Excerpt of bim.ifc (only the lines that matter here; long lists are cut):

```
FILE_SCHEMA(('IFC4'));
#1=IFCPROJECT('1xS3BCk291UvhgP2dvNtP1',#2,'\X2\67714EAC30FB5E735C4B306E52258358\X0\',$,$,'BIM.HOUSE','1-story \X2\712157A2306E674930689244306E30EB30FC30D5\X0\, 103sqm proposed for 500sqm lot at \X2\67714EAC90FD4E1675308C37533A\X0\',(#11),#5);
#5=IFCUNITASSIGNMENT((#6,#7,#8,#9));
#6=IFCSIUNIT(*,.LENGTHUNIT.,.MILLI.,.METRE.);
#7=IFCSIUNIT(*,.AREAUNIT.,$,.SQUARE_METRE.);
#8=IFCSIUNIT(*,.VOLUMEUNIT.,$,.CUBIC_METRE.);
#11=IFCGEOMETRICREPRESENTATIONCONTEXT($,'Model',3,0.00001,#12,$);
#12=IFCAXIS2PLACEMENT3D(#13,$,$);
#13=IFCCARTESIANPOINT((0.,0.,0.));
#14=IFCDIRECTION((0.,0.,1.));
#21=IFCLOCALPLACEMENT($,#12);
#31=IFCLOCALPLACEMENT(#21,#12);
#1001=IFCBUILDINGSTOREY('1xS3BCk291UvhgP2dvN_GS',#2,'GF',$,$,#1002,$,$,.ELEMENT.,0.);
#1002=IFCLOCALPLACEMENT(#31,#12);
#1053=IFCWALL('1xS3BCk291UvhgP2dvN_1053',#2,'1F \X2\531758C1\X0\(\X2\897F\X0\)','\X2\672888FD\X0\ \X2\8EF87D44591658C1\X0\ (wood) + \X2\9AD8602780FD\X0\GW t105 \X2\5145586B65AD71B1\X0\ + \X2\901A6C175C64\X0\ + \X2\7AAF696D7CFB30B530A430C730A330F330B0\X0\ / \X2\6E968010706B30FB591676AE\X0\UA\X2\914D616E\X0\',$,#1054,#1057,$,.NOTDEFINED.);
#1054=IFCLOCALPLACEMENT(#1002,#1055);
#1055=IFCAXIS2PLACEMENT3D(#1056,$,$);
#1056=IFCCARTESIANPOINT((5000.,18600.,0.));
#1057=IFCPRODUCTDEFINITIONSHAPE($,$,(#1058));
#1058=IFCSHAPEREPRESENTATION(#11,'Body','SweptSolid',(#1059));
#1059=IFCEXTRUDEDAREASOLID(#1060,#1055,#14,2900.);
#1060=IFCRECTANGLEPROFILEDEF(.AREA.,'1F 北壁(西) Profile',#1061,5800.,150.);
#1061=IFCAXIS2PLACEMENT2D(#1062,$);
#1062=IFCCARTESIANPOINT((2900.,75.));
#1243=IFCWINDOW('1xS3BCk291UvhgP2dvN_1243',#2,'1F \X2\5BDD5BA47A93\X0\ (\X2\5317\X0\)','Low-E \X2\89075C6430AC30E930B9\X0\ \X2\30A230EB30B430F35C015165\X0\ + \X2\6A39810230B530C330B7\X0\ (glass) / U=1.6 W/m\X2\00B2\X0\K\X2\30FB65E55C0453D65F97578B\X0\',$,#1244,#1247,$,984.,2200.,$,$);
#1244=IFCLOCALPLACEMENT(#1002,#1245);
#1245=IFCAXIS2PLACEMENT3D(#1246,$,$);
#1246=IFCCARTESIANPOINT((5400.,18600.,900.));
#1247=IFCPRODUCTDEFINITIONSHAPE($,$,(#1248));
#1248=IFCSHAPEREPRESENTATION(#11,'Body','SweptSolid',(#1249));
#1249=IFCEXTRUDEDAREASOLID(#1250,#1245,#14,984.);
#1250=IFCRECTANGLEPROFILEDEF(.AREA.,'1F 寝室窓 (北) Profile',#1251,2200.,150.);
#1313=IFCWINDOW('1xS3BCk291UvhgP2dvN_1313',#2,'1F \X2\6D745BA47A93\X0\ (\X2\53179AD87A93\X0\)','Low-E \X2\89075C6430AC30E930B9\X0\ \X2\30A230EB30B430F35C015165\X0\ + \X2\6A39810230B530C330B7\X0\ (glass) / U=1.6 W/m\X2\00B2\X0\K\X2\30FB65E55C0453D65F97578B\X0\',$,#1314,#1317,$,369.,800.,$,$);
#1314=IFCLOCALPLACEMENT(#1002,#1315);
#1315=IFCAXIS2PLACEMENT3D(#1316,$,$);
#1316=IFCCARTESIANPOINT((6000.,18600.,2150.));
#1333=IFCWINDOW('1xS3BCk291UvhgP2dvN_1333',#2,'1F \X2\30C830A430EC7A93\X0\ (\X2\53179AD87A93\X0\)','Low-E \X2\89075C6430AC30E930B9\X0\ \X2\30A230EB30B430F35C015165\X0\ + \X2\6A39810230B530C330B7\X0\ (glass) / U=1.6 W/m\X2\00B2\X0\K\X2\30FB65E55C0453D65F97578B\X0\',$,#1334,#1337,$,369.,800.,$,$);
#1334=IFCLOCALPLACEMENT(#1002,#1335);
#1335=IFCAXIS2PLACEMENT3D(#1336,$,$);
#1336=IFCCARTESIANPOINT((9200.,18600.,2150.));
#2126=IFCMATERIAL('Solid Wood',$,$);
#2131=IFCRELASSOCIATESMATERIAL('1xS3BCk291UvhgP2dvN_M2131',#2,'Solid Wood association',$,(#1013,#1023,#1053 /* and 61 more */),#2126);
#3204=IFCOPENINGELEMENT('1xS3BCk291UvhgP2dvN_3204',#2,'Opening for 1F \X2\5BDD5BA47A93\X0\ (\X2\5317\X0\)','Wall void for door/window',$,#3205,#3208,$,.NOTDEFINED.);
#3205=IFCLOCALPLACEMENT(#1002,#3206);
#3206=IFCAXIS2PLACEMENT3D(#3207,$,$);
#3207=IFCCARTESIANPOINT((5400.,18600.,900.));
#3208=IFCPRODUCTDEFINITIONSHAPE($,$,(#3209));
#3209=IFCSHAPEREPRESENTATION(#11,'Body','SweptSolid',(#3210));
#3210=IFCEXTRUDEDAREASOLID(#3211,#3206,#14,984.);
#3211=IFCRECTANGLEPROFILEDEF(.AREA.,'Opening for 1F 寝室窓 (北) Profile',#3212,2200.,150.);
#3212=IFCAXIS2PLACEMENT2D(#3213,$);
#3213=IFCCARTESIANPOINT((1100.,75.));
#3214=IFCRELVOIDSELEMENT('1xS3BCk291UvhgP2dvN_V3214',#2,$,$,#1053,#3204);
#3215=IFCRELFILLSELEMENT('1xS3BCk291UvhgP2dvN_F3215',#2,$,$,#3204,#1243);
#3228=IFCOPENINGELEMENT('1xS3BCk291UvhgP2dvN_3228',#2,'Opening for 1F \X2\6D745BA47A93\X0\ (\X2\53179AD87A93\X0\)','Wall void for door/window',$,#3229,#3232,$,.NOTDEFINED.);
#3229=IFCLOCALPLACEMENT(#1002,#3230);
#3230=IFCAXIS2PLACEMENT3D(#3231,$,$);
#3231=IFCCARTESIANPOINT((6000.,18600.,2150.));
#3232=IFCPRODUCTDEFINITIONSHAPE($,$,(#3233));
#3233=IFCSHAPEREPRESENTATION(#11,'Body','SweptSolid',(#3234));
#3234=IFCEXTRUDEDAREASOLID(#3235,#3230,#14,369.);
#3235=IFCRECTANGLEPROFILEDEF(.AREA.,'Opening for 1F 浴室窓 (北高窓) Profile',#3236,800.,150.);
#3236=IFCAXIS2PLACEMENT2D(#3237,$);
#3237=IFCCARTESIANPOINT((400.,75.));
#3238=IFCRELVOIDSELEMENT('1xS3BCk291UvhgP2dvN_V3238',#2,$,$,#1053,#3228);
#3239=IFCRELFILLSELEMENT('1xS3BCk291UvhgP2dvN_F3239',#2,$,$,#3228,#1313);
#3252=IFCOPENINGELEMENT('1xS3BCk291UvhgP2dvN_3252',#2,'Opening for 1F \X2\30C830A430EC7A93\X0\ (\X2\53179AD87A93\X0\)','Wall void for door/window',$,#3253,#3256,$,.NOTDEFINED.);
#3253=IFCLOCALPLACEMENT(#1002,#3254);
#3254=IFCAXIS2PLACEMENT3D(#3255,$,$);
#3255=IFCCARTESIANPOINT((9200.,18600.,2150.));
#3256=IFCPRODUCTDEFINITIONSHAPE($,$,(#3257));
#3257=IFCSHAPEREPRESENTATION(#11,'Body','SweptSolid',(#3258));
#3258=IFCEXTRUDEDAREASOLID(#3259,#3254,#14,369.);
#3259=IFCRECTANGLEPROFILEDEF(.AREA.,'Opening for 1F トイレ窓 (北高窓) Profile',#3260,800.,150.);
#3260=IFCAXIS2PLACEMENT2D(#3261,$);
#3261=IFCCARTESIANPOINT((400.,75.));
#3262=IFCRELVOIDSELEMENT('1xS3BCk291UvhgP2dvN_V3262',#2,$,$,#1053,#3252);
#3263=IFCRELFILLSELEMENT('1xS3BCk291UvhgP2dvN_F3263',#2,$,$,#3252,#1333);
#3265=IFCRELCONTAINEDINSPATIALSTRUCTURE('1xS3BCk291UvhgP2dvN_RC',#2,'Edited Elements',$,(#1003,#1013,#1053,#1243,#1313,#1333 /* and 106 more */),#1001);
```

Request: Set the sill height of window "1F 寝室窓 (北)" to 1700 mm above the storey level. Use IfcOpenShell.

```python
import numpy as np
import ifcopenshell
import ifcopenshell.api.geometry
import ifcopenshell.geom
import ifcopenshell.util.element
import ifcopenshell.util.placement
import ifcopenshell.util.shape
import ifcopenshell.util.unit

model = ifcopenshell.open("bim.ifc")
unit_scale = ifcopenshell.util.unit.calculate_unit_scale(model)

window = model.by_id(1243)
opening = window.FillsVoids[0].RelatingOpeningElement
storey = ifcopenshell.util.element.get_container(window, ifc_class="IfcBuildingStorey")
level = ifcopenshell.util.placement.get_local_placement(storey.ObjectPlacement)[2, 3]

# The opening's origin need not be at the sill, so measure its lowest point.
shape = ifcopenshell.geom.create_shape(ifcopenshell.geom.settings(), opening)
bottom = ifcopenshell.util.shape.get_shape_bottom_elevation(shape, shape.geometry) / unit_scale
dz = level + 1.7 / unit_scale - bottom

shift = np.array([0.0, 0.0, dz])
# The window is not placed relative to its opening, so move both.
for product in (opening, window):
    matrix = ifcopenshell.util.placement.get_local_placement(product.ObjectPlacement)
    matrix[:3, 3] += shift
    ifcopenshell.api.geometry.edit_object_placement(model, product=product, matrix=matrix, is_si=False)

print(f"moved by {dz * unit_scale:+.3f} m")

model.write("bim-out.ifc")
```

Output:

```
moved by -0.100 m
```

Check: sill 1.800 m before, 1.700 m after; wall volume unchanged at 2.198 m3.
